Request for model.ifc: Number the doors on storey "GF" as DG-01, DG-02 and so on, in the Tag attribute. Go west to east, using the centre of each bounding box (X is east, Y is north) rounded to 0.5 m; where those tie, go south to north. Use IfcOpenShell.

First a look at what the model holds.

```python
import ifcopenshell
import ifcopenshell.util.element
import ifcopenshell.util.placement

model = ifcopenshell.open("model.ifc")
print(model.schema)
storey = next(s for s in model.by_type("IfcBuildingStorey") if s.Name == "GF")
doors = [e for e in ifcopenshell.util.element.get_decomposition(storey) if e.is_a("IfcDoor")]
for e in sorted(doors, key=lambda e: e.id()):
    origin = ifcopenshell.util.placement.get_local_placement(e.ObjectPlacement)[:3, 3]
    print(e.id(), e.Tag, e.Name, origin.round(2) + 0.0, sep=" | ")
```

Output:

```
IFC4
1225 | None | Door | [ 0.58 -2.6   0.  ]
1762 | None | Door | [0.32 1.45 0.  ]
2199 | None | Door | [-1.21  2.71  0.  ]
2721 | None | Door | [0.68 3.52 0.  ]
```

```python
import ifcopenshell
import ifcopenshell.geom
import ifcopenshell.util.element
import ifcopenshell.util.shape

model = ifcopenshell.open("model.ifc")
settings = ifcopenshell.geom.settings()
settings.set("use-world-coords", True)


def centre(element):
    shape = ifcopenshell.geom.create_shape(settings, element)
    return ifcopenshell.util.shape.get_bbox_centroid(shape.geometry)


storey = next(s for s in model.by_type("IfcBuildingStorey") if s.Name == "GF")
doors = [e for e in ifcopenshell.util.element.get_decomposition(storey) if e.is_a("IfcDoor")]

# Insertion points can sit at a corner or the storey origin, so sort by the geometry (in metres).
centres = {e: centre(e) for e in doors}
doors.sort(key=lambda e: (round(centres[e][0] / 0.5), centres[e][1]))

for i, e in enumerate(doors, start=1):
    number = f"DG-{i:02d}"
    e.Tag = number
    print(e.id(), number)

model.write("model-out.ifc")
```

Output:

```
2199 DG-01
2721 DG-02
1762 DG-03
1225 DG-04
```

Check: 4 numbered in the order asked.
